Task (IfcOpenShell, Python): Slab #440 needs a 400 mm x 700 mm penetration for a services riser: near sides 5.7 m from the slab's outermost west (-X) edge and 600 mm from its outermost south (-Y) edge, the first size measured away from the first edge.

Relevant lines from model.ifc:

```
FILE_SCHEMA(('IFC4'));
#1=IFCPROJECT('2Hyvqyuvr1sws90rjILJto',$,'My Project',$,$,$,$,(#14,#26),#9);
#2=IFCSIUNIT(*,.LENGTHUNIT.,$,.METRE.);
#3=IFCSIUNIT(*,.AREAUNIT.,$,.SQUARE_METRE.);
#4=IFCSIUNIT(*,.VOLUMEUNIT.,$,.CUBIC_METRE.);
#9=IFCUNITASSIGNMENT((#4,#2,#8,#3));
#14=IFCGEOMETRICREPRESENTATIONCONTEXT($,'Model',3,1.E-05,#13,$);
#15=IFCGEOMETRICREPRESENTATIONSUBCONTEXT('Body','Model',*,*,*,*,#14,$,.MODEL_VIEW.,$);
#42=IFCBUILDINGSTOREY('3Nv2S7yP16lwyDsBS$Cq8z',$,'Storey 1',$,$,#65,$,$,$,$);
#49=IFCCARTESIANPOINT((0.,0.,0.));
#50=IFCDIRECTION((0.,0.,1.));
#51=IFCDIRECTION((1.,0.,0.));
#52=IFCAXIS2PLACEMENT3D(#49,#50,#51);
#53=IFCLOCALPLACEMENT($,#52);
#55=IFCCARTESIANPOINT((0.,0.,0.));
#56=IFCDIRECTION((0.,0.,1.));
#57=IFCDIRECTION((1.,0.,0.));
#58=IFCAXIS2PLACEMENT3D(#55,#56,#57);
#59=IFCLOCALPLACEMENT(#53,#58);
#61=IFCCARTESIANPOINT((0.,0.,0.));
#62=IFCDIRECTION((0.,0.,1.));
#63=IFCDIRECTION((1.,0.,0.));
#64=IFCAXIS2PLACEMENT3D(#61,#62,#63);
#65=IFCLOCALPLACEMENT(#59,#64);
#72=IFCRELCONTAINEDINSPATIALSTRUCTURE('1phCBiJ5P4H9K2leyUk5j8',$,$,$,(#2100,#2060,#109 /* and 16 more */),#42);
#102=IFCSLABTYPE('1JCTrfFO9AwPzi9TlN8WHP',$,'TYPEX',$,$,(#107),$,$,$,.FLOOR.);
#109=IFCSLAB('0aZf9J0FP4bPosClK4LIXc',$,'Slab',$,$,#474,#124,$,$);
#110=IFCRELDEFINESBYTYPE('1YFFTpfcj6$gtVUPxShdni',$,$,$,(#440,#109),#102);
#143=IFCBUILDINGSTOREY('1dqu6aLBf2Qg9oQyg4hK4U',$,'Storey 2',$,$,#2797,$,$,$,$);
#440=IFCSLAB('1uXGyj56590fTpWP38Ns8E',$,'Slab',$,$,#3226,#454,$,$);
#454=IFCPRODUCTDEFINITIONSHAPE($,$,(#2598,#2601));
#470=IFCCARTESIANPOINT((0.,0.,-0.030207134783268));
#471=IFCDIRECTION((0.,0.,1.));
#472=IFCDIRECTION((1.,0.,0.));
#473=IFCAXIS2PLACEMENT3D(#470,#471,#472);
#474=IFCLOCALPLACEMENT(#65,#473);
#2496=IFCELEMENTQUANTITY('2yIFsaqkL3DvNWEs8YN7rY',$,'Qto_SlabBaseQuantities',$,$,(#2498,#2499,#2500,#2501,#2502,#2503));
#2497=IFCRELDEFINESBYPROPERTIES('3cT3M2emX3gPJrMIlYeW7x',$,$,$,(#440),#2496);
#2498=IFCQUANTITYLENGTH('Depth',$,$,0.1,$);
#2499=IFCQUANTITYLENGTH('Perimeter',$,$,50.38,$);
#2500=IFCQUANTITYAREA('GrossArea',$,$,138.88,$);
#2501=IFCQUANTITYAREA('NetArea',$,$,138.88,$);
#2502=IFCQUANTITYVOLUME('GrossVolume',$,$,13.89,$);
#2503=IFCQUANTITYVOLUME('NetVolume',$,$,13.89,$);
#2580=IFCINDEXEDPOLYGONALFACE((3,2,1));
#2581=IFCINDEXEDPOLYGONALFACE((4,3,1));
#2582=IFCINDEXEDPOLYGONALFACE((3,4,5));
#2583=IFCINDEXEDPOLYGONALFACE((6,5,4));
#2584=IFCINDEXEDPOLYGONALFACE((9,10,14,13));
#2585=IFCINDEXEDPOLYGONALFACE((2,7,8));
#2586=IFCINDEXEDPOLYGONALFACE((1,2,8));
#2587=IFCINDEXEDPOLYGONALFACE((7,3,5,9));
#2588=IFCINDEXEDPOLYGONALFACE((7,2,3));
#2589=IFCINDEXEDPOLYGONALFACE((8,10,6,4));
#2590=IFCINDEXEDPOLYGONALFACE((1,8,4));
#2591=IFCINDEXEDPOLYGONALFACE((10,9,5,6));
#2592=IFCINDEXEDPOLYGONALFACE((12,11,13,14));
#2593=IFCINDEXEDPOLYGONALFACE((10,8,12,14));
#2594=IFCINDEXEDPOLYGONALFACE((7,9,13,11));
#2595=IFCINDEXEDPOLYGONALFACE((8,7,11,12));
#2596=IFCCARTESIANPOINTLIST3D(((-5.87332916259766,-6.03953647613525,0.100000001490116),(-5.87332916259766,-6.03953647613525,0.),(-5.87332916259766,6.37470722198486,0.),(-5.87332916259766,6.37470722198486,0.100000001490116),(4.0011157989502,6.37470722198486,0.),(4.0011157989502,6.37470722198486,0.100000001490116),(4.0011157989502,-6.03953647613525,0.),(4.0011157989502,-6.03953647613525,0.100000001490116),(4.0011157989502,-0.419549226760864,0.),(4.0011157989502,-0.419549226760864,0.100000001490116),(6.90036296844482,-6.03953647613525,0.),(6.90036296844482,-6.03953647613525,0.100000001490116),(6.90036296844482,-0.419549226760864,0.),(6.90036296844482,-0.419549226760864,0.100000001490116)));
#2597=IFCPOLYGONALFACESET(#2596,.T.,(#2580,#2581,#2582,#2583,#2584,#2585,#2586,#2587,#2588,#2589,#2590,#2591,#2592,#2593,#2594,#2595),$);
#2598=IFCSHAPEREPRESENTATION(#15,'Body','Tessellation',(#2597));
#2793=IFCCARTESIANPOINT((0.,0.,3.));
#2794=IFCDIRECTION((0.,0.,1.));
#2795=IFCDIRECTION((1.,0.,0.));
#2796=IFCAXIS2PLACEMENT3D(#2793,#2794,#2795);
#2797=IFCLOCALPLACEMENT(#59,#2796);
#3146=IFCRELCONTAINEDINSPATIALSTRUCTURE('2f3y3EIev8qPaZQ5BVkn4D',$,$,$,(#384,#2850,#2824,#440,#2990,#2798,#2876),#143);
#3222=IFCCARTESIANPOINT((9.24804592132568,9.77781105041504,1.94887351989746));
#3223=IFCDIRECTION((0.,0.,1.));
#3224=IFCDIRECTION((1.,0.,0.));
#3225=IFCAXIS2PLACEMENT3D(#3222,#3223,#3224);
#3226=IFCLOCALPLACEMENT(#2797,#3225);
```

```python
import numpy as np
import ifcopenshell
import ifcopenshell.api.feature
import ifcopenshell.api.geometry
import ifcopenshell.api.pset
import ifcopenshell.api.root
import ifcopenshell.geom
import ifcopenshell.util.element
import ifcopenshell.util.placement
import ifcopenshell.util.representation
import ifcopenshell.util.shape
import ifcopenshell.util.unit

model = ifcopenshell.open("model.ifc")
unit_scale = ifcopenshell.util.unit.calculate_unit_scale(model)
area_scale = ifcopenshell.util.unit.calculate_unit_scale(model, "AREAUNIT")
volume_scale = ifcopenshell.util.unit.calculate_unit_scale(model, "VOLUMEUNIT")
settings = ifcopenshell.geom.settings()


def volume(element):
    """Net volume in cubic metres, openings subtracted."""
    shape = ifcopenshell.geom.create_shape(settings, element)
    return ifcopenshell.util.shape.get_volume(shape.geometry)


slab = model.by_guid("1uXGyj56590fTpWP38Ns8E")
before = volume(slab)

# Extent in the slab's own axes, in metres. The edges named are its -X and -Y sides.
slab_shape = ifcopenshell.geom.create_shape(settings, slab)
vertices = ifcopenshell.util.shape.get_vertices(slab_shape.geometry)
x_min, y_min, bottom = vertices.min(axis=0)
top = vertices[:, 2].max()

opening = ifcopenshell.api.root.create_entity(model, ifc_class="IfcOpeningElement", name="Services riser opening", predefined_type="OPENING")
context = ifcopenshell.util.representation.get_context(model, "Model", "Body", "MODEL_VIEW")
width, depth = 0.4, 0.7
outline = [(0.0, 0.0), (width, 0.0), (width, depth), (0.0, depth), (0.0, 0.0)]
# Overshoot both faces by 50 mm so the cut is clean.
shape = ifcopenshell.api.geometry.add_slab_representation(
    model, context=context, depth=top - bottom + 0.1, polyline=outline
)
ifcopenshell.api.geometry.assign_representation(model, product=opening, representation=shape)

matrix = ifcopenshell.util.placement.get_local_placement(slab.ObjectPlacement)
matrix[:, 3] = matrix @ np.append(np.array([x_min + 5.7, y_min + 0.6, bottom - 0.05]) / unit_scale, 1.0)
ifcopenshell.api.geometry.edit_object_placement(model, product=opening, matrix=matrix, is_si=False)
ifcopenshell.api.feature.add_feature(model, feature=opening, element=slab)

after = volume(slab)

# Update the slab's stored quantities.
qto = model.by_id(ifcopenshell.util.element.get_pset(slab, "Qto_SlabBaseQuantities", should_inherit=False)["id"])
ifcopenshell.api.pset.edit_qto(model, qto=qto, properties={
    "NetArea": after / (top - bottom) / area_scale,
    "NetVolume": after / volume_scale,
})

print(f"slab volume {before:.3f} -> {after:.3f} m3")

model.write("model_updated.ifc")
```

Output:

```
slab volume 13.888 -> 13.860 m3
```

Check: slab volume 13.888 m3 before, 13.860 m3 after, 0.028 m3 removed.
